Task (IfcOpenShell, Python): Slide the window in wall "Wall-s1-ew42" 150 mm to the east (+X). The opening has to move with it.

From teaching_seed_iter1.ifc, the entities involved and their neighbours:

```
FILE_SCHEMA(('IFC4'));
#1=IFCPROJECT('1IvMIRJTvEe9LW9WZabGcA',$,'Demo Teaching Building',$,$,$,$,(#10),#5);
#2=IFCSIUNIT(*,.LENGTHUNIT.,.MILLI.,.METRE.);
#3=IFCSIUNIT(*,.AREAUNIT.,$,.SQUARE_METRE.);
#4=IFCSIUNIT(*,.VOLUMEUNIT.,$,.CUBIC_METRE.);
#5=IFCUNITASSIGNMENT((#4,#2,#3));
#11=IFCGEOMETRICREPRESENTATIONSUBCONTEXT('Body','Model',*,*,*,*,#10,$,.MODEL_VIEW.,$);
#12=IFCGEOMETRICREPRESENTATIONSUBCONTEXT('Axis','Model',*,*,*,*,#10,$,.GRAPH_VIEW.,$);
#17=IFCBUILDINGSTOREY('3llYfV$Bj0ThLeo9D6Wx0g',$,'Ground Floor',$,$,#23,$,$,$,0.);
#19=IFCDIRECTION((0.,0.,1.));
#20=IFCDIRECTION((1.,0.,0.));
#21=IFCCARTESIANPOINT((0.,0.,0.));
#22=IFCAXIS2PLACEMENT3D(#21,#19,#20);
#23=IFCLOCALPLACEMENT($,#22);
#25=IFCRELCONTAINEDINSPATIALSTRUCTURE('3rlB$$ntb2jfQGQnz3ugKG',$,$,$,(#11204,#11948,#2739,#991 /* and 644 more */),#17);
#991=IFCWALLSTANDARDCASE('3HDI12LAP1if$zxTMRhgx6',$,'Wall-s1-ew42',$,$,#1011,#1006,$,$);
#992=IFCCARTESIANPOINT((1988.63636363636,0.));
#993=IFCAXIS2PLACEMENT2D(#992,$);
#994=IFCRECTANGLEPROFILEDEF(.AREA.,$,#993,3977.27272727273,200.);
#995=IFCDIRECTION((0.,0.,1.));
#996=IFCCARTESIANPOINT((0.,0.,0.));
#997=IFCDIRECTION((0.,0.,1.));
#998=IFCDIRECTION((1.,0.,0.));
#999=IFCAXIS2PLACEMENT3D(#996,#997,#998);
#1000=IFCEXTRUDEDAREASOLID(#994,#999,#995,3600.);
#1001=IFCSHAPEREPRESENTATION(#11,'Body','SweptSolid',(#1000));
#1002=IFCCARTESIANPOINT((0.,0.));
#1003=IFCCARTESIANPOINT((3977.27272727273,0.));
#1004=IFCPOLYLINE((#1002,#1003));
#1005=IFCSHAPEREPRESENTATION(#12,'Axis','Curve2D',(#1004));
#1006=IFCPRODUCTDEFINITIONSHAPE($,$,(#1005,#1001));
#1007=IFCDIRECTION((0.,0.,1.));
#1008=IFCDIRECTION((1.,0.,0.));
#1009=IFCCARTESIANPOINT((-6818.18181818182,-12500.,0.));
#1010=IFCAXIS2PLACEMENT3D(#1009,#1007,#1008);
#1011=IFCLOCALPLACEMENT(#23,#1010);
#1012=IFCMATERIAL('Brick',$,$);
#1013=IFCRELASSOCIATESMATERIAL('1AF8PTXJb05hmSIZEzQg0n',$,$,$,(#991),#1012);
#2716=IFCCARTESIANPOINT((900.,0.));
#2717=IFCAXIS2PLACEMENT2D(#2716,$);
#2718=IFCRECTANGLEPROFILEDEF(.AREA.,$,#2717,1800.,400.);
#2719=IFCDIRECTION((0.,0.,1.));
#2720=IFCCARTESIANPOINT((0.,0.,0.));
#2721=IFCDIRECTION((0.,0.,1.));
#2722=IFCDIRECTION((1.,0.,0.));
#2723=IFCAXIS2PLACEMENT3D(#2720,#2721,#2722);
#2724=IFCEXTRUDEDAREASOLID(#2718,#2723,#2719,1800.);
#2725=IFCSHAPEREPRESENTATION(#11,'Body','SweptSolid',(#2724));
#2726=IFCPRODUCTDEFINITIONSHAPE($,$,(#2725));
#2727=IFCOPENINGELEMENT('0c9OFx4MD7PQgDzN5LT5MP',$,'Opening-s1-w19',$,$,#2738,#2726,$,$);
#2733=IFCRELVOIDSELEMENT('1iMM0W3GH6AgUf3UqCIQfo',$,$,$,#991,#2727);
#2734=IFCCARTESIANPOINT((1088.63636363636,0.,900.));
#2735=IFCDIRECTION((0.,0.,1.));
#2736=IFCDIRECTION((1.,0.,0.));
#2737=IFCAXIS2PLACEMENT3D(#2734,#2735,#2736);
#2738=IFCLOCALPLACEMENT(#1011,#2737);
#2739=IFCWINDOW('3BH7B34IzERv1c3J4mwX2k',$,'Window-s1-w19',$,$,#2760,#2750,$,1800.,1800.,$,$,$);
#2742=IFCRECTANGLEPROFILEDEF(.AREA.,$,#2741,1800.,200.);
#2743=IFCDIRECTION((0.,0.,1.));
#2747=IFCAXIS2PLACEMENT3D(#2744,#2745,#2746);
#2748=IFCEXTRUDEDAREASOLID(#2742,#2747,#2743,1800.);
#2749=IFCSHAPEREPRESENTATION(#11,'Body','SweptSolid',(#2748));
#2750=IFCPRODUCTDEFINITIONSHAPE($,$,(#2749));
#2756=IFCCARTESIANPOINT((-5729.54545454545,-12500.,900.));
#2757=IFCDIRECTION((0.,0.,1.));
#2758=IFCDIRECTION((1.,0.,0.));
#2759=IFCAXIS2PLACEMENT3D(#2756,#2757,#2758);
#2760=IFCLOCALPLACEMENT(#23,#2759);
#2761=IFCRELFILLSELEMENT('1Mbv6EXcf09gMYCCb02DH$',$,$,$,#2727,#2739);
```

```python
import ifcopenshell
import ifcopenshell.api.geometry
import ifcopenshell.util.placement

model = ifcopenshell.open("teaching_seed_iter1.ifc")

window = model.by_guid("3BH7B34IzERv1c3J4mwX2k")
opening = window.FillsVoids[0].RelatingOpeningElement
wall = opening.VoidsElements[0].RelatingBuildingElement

wall_matrix = ifcopenshell.util.placement.get_local_placement(wall.ObjectPlacement)
shift = wall_matrix[:3, 0] * 150.0
before = ifcopenshell.util.placement.get_local_placement(window.ObjectPlacement)[:3, 3].copy()

# The window is not placed relative to its opening, so move both.
for product in (opening, window):
    matrix = ifcopenshell.util.placement.get_local_placement(product.ObjectPlacement)
    matrix[:3, 3] += shift
    ifcopenshell.api.geometry.edit_object_placement(model, product=product, matrix=matrix, is_si=False)

after = ifcopenshell.util.placement.get_local_placement(window.ObjectPlacement)[:3, 3]
print("window moved by", (after - before).round(3) + 0.0)

model.write("teaching_seed_iter1-out.ifc")
```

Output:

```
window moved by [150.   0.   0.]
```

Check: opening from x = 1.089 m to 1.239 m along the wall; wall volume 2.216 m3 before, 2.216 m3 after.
